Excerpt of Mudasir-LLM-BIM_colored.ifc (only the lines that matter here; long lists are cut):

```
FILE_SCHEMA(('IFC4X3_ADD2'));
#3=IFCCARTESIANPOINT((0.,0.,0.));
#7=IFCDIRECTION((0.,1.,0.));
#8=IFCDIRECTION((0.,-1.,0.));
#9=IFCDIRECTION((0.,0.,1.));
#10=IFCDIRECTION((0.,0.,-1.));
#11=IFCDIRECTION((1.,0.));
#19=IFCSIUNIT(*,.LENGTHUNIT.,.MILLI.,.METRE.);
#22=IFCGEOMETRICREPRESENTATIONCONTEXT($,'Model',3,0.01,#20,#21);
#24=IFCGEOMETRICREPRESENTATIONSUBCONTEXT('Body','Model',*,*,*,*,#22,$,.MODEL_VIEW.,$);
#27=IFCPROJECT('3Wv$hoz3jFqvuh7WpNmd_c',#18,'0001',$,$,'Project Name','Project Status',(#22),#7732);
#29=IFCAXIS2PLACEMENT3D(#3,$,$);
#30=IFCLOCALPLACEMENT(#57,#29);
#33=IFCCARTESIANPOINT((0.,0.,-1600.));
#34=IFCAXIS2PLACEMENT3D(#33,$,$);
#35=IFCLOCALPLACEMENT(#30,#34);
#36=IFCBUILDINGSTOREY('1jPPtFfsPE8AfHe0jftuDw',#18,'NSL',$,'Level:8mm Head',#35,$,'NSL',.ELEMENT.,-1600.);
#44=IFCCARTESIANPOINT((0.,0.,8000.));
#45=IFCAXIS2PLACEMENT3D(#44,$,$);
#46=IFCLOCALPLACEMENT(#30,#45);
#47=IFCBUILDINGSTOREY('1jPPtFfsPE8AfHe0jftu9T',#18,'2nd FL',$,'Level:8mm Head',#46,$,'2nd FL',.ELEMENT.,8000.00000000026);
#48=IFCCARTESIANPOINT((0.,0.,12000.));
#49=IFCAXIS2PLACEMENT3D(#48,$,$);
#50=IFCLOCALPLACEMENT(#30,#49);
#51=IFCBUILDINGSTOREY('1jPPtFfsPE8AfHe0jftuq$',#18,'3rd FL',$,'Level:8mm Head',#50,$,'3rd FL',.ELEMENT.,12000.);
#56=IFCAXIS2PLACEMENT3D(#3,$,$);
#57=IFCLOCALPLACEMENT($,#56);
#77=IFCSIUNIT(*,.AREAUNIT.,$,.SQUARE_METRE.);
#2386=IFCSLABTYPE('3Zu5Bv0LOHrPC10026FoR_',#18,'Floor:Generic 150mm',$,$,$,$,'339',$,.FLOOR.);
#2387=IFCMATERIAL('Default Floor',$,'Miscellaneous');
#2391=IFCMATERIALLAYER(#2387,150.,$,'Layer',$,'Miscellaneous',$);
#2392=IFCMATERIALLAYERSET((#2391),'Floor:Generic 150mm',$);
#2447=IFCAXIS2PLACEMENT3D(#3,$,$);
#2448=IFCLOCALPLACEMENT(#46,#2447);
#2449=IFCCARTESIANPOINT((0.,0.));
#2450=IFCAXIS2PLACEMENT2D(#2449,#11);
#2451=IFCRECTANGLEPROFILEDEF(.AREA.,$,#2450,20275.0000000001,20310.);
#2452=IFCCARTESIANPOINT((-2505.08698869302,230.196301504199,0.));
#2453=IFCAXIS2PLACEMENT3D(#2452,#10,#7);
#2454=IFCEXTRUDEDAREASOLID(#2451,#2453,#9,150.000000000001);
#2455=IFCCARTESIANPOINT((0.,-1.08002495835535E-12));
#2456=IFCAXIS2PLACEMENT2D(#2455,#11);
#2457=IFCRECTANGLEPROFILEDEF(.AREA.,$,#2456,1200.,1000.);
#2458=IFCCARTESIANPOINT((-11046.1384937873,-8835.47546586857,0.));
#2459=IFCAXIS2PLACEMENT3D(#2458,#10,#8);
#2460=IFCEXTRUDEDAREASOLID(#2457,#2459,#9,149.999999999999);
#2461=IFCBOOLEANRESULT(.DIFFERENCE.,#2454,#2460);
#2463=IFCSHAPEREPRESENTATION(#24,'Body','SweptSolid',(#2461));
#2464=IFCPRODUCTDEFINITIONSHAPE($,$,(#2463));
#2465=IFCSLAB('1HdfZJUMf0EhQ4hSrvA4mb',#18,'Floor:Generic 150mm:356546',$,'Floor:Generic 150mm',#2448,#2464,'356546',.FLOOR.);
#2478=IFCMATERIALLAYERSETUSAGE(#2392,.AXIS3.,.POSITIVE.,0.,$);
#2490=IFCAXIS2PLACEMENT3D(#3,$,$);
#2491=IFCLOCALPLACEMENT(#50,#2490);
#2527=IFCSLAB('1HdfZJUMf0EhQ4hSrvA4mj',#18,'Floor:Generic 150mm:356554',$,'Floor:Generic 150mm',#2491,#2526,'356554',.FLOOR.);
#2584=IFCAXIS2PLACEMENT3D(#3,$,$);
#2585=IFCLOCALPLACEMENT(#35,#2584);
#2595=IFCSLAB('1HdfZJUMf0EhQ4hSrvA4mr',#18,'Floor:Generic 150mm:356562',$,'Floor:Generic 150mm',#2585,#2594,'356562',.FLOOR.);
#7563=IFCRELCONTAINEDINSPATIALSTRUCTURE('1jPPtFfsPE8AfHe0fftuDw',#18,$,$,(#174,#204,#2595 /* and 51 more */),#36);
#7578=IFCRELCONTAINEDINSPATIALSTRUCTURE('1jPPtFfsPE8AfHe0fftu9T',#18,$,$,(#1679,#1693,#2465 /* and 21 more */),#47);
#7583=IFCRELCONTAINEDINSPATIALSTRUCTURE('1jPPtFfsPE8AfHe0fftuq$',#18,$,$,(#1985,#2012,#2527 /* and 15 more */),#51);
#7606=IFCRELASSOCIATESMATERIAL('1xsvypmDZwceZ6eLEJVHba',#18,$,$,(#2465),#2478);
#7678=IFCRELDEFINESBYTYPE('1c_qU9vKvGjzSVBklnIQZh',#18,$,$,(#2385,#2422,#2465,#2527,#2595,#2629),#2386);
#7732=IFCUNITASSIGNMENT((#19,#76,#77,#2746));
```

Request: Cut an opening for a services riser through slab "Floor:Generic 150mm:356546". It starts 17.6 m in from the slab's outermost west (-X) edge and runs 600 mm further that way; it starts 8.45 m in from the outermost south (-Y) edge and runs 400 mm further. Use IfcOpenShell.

```python
import numpy as np
import ifcopenshell
import ifcopenshell.api.feature
import ifcopenshell.api.geometry
import ifcopenshell.api.root
import ifcopenshell.geom
import ifcopenshell.util.placement
import ifcopenshell.util.representation
import ifcopenshell.util.shape
import ifcopenshell.util.unit

model = ifcopenshell.open("Mudasir-LLM-BIM_colored.ifc")
unit_scale = ifcopenshell.util.unit.calculate_unit_scale(model)
settings = ifcopenshell.geom.settings()


def volume(element):
    """Net volume in cubic metres, openings subtracted."""
    shape = ifcopenshell.geom.create_shape(settings, element)
    return ifcopenshell.util.shape.get_volume(shape.geometry)


slab = model.by_guid("1HdfZJUMf0EhQ4hSrvA4mb")
before = volume(slab)

# Extent in the slab's own axes, in metres. The edges named are its -X and -Y sides.
slab_shape = ifcopenshell.geom.create_shape(settings, slab)
vertices = ifcopenshell.util.shape.get_vertices(slab_shape.geometry)
x_min, y_min, bottom = vertices.min(axis=0)
top = vertices[:, 2].max()

opening = ifcopenshell.api.root.create_entity(model, ifc_class="IfcOpeningElement", name="Services riser opening", predefined_type="OPENING")
context = ifcopenshell.util.representation.get_context(model, "Model", "Body", "MODEL_VIEW")
width, depth = 0.6, 0.4
outline = [(0.0, 0.0), (width, 0.0), (width, depth), (0.0, depth), (0.0, 0.0)]
# Overshoot both faces by 50 mm so the cut is clean.
shape = ifcopenshell.api.geometry.add_slab_representation(
    model, context=context, depth=top - bottom + 0.1, polyline=outline
)
ifcopenshell.api.geometry.assign_representation(model, product=opening, representation=shape)

matrix = ifcopenshell.util.placement.get_local_placement(slab.ObjectPlacement)
matrix[:, 3] = matrix @ np.append(np.array([x_min + 17.6, y_min + 8.45, bottom - 0.05]) / unit_scale, 1.0)
ifcopenshell.api.geometry.edit_object_placement(model, product=opening, matrix=matrix, is_si=False)
ifcopenshell.api.feature.add_feature(model, feature=opening, element=slab)

after = volume(slab)

print(f"slab volume {before:.3f} -> {after:.3f} m3")

model.write("Mudasir-LLM-BIM_colored_rev.ifc")
```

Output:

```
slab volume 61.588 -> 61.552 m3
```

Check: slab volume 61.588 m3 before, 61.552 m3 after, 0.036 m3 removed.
